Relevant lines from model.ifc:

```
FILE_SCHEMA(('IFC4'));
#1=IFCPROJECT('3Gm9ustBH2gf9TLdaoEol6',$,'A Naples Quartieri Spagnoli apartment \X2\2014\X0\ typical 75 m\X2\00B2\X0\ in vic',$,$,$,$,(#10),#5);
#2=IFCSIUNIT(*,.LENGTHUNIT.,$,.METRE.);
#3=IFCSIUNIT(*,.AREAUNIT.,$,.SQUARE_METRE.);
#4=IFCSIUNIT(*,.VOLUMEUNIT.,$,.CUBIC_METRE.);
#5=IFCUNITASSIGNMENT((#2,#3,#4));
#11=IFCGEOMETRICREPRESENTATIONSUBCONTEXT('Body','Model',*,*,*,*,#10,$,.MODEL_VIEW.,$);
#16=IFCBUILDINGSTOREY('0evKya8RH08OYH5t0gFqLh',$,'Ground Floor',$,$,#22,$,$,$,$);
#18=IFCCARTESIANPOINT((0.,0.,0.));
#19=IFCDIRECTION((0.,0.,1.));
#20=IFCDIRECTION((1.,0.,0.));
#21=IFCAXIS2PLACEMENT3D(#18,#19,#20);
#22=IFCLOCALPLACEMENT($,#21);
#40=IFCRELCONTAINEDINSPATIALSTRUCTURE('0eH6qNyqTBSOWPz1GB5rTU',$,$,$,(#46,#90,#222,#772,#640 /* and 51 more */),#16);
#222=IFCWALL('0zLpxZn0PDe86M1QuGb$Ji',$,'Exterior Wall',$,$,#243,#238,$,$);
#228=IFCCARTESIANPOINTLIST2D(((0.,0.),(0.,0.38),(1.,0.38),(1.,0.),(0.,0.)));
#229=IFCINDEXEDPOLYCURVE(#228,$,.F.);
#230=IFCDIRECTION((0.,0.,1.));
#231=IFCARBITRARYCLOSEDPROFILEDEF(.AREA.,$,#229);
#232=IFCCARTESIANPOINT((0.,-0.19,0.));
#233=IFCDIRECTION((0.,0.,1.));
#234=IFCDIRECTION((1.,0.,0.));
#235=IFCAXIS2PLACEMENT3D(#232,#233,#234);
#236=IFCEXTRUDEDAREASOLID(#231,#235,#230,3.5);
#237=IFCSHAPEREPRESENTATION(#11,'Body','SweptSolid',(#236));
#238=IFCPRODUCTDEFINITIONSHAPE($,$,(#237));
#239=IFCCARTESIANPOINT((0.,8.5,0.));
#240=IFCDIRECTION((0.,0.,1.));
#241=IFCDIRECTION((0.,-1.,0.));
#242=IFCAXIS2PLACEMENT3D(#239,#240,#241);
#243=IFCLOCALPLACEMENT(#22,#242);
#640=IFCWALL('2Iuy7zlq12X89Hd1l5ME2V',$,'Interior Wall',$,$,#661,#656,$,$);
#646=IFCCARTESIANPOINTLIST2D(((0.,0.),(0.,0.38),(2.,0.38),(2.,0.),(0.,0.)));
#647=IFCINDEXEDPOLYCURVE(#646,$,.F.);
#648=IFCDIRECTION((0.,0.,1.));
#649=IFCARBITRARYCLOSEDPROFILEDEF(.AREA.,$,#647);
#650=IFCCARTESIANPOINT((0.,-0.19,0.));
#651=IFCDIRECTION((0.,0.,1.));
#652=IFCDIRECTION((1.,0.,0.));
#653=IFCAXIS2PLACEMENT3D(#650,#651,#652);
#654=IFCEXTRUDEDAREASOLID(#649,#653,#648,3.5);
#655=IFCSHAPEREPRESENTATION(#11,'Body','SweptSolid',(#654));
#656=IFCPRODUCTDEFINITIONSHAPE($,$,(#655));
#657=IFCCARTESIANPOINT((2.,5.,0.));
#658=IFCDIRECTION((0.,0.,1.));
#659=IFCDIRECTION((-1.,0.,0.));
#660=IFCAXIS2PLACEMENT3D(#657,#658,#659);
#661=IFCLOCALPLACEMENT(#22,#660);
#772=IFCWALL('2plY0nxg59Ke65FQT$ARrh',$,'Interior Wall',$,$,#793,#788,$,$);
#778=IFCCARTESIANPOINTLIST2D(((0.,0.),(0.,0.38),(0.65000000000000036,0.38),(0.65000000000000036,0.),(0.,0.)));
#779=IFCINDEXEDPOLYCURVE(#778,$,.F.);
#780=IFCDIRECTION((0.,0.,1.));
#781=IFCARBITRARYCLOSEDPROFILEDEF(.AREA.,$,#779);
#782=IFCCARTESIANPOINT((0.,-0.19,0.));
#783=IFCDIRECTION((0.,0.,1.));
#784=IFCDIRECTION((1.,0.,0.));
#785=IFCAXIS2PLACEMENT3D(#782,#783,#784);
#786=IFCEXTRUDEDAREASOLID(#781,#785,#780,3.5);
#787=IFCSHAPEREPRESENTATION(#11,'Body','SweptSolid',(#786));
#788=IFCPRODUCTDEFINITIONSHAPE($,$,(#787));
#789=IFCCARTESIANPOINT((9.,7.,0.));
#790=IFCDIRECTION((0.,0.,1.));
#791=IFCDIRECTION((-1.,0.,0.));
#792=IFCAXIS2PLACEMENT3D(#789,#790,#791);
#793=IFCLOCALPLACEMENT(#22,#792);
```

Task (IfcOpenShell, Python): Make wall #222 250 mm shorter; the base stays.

```python
import ifcopenshell
import ifcopenshell.geom
import ifcopenshell.util.representation
import ifcopenshell.util.shape
import ifcopenshell.util.unit

model = ifcopenshell.open("model.ifc")
unit_scale = ifcopenshell.util.unit.calculate_unit_scale(model)
settings = ifcopenshell.geom.settings()


def volume(element):
    """Net volume in cubic metres, openings subtracted."""
    shape = ifcopenshell.geom.create_shape(settings, element)
    return ifcopenshell.util.shape.get_volume(shape.geometry)


wall = model.by_id(222)
before = volume(wall)

body = ifcopenshell.util.representation.get_representation(wall, "Model", "Body")
solid = body.Items[0]
old_height = solid.Depth
solid.Depth -= 0.25 / unit_scale
after = volume(wall)

print(f"height {old_height:g} -> {solid.Depth:g}, volume {before:.3f} -> {after:.3f} m3")

model.write("model_v2.ifc")
```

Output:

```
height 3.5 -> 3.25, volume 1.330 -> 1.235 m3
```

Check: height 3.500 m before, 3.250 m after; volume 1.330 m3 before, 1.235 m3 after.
